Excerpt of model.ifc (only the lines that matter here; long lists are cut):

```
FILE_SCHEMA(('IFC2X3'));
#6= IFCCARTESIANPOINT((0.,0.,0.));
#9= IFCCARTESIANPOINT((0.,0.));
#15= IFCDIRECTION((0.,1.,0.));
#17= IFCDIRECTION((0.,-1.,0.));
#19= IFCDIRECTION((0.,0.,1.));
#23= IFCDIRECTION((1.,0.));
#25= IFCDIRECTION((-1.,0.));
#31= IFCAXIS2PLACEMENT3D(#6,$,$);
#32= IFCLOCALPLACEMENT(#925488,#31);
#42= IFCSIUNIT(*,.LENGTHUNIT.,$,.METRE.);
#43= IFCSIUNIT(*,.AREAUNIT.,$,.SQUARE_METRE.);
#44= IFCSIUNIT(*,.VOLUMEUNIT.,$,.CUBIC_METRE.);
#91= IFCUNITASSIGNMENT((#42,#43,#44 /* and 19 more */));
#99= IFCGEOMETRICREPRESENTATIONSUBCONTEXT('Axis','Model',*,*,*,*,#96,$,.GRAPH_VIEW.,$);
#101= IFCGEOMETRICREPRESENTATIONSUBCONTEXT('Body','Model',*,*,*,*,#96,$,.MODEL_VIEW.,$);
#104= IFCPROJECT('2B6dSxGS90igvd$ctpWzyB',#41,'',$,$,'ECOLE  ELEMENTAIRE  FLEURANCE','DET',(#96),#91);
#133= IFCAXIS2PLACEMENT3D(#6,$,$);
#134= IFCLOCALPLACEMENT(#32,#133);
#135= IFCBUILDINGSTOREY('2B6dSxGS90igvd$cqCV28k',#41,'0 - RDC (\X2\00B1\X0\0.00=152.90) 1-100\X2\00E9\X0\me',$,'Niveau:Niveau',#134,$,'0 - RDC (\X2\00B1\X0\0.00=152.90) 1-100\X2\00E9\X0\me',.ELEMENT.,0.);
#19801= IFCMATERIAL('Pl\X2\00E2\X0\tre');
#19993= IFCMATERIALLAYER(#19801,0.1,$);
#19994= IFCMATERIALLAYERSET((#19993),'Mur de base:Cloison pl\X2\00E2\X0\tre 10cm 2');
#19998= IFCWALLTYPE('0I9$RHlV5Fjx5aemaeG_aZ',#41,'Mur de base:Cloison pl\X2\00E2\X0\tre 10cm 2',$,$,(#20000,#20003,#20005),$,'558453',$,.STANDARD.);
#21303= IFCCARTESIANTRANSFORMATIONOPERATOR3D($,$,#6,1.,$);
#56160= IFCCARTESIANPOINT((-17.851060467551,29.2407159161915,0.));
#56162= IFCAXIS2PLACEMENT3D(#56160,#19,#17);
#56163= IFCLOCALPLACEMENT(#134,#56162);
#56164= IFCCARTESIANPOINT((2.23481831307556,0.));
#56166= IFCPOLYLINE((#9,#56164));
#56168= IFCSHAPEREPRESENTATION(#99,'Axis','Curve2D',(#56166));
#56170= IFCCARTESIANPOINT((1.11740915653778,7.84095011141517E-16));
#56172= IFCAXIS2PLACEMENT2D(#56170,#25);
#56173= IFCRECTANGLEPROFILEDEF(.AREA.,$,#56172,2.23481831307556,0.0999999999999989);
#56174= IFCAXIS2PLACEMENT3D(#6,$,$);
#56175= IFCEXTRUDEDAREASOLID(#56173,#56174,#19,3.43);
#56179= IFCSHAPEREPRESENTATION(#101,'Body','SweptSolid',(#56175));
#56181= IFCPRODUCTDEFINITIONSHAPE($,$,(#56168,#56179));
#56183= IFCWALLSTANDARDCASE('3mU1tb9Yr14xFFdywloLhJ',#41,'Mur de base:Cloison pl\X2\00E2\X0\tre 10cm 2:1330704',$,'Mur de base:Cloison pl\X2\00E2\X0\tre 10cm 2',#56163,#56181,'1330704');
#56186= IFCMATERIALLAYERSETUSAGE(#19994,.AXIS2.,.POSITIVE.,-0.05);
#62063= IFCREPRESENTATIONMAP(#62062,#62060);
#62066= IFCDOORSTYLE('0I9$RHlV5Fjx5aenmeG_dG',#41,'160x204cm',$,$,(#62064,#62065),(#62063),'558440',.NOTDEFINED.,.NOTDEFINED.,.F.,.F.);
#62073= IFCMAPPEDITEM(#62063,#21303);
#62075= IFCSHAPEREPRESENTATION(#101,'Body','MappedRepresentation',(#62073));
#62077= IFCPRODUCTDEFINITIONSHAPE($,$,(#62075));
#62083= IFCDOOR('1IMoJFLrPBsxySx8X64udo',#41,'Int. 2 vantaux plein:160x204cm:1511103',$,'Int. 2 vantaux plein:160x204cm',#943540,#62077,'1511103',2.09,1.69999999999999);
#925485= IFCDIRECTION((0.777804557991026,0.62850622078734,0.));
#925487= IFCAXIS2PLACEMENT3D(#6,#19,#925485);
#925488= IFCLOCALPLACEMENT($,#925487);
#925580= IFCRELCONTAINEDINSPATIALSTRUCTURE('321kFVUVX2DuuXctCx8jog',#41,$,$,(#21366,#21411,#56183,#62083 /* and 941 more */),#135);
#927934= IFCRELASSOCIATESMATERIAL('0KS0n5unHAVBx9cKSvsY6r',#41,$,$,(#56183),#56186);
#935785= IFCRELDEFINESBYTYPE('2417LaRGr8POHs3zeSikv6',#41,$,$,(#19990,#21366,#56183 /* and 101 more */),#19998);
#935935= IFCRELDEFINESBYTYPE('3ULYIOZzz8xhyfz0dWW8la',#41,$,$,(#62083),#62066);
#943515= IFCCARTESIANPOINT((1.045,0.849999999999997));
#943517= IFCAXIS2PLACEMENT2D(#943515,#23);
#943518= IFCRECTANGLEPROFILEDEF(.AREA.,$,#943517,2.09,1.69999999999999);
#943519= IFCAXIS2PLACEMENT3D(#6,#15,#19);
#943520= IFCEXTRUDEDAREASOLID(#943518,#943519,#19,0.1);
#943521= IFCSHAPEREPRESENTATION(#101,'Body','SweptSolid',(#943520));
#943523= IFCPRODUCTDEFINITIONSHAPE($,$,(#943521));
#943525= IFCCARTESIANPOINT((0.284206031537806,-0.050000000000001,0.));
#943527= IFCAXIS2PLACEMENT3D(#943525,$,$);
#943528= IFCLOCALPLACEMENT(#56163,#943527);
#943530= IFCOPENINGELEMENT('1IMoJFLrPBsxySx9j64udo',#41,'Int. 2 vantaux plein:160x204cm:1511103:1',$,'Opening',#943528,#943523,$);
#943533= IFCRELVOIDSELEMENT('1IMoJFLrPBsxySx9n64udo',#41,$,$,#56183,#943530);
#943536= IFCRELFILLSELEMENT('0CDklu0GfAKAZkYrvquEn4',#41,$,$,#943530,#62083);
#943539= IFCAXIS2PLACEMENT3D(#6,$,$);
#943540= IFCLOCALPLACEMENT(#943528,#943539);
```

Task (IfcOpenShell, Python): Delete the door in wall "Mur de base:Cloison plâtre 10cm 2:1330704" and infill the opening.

```python
import ifcopenshell
import ifcopenshell.api.feature
import ifcopenshell.api.root
import ifcopenshell.geom
import ifcopenshell.util.shape

model = ifcopenshell.open("model.ifc")
settings = ifcopenshell.geom.settings()


def volume(element):
    """Net volume in cubic metres, openings subtracted."""
    shape = ifcopenshell.geom.create_shape(settings, element)
    return ifcopenshell.util.shape.get_volume(shape.geometry)


door = model.by_guid("1IMoJFLrPBsxySx8X64udo")
opening = door.FillsVoids[0].RelatingOpeningElement
wall = opening.VoidsElements[0].RelatingBuildingElement
before = volume(wall)

ifcopenshell.api.root.remove_product(model, product=door)
ifcopenshell.api.feature.remove_feature(model, feature=opening)

after = volume(wall)

print(f"wall volume {before:.3f} -> {after:.3f} m3")

model.write("model_rev.ifc")
```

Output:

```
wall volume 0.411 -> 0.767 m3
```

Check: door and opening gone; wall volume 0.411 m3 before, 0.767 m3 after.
